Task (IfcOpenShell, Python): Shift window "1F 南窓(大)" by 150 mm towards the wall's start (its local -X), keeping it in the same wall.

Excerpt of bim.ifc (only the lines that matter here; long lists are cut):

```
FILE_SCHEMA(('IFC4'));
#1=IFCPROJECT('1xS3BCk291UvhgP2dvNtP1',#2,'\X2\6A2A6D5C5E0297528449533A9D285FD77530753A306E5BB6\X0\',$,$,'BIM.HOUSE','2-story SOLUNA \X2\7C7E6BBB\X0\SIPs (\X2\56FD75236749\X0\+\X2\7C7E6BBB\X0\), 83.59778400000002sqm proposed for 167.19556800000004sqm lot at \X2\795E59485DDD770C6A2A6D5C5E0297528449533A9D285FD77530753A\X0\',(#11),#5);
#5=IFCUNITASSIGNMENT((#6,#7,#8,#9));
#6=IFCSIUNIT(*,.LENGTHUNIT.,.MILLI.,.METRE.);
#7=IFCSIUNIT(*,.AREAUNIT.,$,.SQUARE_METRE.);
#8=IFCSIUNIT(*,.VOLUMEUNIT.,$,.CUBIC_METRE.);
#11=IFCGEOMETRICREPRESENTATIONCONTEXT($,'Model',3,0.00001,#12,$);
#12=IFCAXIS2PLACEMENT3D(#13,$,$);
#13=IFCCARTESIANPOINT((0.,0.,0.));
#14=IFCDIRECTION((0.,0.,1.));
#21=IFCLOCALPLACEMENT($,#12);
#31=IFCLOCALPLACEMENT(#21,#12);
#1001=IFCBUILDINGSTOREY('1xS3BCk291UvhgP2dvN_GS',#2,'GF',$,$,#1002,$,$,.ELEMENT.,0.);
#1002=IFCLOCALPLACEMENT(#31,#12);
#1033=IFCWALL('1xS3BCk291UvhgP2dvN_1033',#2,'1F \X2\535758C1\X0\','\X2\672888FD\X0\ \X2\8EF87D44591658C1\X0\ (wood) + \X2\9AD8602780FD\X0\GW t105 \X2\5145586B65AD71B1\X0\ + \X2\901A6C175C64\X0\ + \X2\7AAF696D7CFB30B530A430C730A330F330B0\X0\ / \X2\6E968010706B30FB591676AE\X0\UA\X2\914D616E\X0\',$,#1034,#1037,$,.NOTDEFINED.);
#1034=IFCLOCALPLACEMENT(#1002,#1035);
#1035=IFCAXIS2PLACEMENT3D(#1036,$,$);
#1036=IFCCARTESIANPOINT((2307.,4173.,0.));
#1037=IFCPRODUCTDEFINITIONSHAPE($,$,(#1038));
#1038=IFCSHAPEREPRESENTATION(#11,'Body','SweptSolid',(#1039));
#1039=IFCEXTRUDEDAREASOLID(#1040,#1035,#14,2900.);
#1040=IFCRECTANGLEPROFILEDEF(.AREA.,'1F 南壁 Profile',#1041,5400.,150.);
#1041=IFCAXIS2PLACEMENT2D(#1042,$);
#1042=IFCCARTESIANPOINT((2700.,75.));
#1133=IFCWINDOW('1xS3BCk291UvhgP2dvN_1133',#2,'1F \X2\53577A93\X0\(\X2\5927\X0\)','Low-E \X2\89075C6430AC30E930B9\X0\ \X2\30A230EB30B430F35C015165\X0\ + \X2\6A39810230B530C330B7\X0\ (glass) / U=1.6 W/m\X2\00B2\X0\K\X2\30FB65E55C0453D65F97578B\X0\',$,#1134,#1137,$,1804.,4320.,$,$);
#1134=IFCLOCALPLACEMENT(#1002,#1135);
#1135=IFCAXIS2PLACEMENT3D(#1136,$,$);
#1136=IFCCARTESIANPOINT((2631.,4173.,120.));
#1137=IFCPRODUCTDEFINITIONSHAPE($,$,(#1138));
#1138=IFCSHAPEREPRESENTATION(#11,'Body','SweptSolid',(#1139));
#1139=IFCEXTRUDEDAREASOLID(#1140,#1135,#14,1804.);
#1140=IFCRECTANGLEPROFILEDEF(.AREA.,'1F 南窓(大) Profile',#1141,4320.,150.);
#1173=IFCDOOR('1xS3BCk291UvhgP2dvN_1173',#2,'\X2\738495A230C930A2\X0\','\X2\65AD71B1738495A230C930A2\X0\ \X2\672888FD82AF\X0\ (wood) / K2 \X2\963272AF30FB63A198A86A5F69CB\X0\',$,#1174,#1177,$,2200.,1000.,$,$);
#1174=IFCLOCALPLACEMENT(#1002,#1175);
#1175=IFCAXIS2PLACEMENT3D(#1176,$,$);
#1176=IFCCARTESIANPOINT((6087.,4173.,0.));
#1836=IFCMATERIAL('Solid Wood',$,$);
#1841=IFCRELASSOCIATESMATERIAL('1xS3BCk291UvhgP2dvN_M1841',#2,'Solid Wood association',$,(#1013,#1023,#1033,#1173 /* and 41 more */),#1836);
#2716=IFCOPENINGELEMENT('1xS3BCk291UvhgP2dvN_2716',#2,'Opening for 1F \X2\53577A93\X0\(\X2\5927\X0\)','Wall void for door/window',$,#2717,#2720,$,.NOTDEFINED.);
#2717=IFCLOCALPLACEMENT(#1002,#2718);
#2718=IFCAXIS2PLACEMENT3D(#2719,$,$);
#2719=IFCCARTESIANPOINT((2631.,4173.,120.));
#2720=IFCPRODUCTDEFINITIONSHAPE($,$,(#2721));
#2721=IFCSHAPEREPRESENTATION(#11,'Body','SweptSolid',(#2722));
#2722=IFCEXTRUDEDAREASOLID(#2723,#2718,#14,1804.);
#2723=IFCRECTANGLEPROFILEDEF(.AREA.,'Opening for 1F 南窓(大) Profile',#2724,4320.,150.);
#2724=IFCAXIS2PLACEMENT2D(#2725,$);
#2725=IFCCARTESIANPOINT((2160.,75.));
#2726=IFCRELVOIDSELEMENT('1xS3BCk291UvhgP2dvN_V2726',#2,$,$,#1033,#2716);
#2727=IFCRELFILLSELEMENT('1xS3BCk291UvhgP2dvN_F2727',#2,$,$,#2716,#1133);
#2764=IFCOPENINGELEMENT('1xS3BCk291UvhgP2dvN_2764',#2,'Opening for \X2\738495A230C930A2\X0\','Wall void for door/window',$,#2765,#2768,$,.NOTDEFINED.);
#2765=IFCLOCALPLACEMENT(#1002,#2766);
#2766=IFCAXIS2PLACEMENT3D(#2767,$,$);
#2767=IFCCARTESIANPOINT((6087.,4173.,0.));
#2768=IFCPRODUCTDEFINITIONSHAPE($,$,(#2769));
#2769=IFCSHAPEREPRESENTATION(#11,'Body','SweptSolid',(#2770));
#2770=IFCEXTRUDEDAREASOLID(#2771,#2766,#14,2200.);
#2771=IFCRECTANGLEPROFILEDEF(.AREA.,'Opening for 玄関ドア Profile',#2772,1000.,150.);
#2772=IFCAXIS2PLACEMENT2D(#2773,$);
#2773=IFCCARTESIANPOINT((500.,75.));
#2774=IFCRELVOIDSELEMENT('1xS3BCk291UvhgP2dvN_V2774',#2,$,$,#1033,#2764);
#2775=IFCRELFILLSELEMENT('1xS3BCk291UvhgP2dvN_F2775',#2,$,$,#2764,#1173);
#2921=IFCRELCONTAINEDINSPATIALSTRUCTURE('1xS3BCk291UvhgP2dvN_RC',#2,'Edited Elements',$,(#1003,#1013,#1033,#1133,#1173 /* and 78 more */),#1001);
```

```python
import ifcopenshell
import ifcopenshell.api.geometry
import ifcopenshell.util.placement
import ifcopenshell.util.unit

model = ifcopenshell.open("bim.ifc")
unit_scale = ifcopenshell.util.unit.calculate_unit_scale(model)

window = model.by_guid("1xS3BCk291UvhgP2dvN_1133")
opening = window.FillsVoids[0].RelatingOpeningElement
wall = opening.VoidsElements[0].RelatingBuildingElement

wall_matrix = ifcopenshell.util.placement.get_local_placement(wall.ObjectPlacement)
shift = wall_matrix[:3, 0] * -0.15 / unit_scale
before = ifcopenshell.util.placement.get_local_placement(window.ObjectPlacement)[:3, 3].copy()

# The window is not placed relative to its opening, so move both.
for product in (opening, window):
    matrix = ifcopenshell.util.placement.get_local_placement(product.ObjectPlacement)
    matrix[:3, 3] += shift
    ifcopenshell.api.geometry.edit_object_placement(model, product=product, matrix=matrix, is_si=False)

after = ifcopenshell.util.placement.get_local_placement(window.ObjectPlacement)[:3, 3]
print("window moved by", (after - before).round(3) + 0.0)

model.write("bim_v2.ifc")
```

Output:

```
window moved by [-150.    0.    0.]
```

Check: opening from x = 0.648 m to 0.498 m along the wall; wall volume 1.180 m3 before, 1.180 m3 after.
